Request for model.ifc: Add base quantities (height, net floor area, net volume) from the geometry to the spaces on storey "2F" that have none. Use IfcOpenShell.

First a look at what the model holds.

```python
import ifcopenshell
import ifcopenshell.util.element
import ifcopenshell.util.unit

model = ifcopenshell.open("model.ifc")
print(model.schema)
for unit_type in ("LENGTHUNIT", "AREAUNIT", "VOLUMEUNIT"):
    print(unit_type, ifcopenshell.util.unit.calculate_unit_scale(model, unit_type))
storey = next(s for s in model.by_type("IfcBuildingStorey") if s.Name == "2F")
spaces = [e for e in ifcopenshell.util.element.get_decomposition(storey) if e.is_a("IfcSpace")]
for e in sorted(spaces, key=lambda e: e.id()):
    print(e.id(), e.is_a(), e.Name, list(ifcopenshell.util.element.get_psets(e, qtos_only=True)), sep=" | ")
```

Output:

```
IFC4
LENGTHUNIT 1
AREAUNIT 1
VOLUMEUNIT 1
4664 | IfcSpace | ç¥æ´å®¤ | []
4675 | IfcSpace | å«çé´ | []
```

```python
import ifcopenshell
import ifcopenshell.api.pset
import ifcopenshell.geom
import ifcopenshell.util.element
import ifcopenshell.util.shape
import ifcopenshell.util.unit

model = ifcopenshell.open("model.ifc")
unit_scale = ifcopenshell.util.unit.calculate_unit_scale(model)
area_scale = ifcopenshell.util.unit.calculate_unit_scale(model, "AREAUNIT")
volume_scale = ifcopenshell.util.unit.calculate_unit_scale(model, "VOLUMEUNIT")
settings = ifcopenshell.geom.settings()

storey = next(s for s in model.by_type("IfcBuildingStorey") if s.Name == "2F")
spaces = [e for e in ifcopenshell.util.element.get_decomposition(storey) if e.is_a("IfcSpace")]

for e in sorted(spaces, key=lambda e: e.id()):
    if ifcopenshell.util.element.get_psets(e, qtos_only=True, should_inherit=False):
        continue
    # Geometry comes back in metres, in the element's own axes.
    shape = ifcopenshell.geom.create_shape(settings, e)
    values = {
        "Height": ifcopenshell.util.shape.get_z(shape.geometry) / unit_scale,
        "NetFloorArea": ifcopenshell.util.shape.get_footprint_area(shape.geometry) / area_scale,
        "NetVolume": ifcopenshell.util.shape.get_volume(shape.geometry) / volume_scale,
    }
    qto = ifcopenshell.api.pset.add_qto(model, product=e, name="Qto_SpaceBaseQuantities")
    ifcopenshell.api.pset.edit_qto(model, qto=qto, properties=values)
    print(e.id(), {k: round(v, 3) for k, v in values.items()})

model.write("model_edited.ifc")
```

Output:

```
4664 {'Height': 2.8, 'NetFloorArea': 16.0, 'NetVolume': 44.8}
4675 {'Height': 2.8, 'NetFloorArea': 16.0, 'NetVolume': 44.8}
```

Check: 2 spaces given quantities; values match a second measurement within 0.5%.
